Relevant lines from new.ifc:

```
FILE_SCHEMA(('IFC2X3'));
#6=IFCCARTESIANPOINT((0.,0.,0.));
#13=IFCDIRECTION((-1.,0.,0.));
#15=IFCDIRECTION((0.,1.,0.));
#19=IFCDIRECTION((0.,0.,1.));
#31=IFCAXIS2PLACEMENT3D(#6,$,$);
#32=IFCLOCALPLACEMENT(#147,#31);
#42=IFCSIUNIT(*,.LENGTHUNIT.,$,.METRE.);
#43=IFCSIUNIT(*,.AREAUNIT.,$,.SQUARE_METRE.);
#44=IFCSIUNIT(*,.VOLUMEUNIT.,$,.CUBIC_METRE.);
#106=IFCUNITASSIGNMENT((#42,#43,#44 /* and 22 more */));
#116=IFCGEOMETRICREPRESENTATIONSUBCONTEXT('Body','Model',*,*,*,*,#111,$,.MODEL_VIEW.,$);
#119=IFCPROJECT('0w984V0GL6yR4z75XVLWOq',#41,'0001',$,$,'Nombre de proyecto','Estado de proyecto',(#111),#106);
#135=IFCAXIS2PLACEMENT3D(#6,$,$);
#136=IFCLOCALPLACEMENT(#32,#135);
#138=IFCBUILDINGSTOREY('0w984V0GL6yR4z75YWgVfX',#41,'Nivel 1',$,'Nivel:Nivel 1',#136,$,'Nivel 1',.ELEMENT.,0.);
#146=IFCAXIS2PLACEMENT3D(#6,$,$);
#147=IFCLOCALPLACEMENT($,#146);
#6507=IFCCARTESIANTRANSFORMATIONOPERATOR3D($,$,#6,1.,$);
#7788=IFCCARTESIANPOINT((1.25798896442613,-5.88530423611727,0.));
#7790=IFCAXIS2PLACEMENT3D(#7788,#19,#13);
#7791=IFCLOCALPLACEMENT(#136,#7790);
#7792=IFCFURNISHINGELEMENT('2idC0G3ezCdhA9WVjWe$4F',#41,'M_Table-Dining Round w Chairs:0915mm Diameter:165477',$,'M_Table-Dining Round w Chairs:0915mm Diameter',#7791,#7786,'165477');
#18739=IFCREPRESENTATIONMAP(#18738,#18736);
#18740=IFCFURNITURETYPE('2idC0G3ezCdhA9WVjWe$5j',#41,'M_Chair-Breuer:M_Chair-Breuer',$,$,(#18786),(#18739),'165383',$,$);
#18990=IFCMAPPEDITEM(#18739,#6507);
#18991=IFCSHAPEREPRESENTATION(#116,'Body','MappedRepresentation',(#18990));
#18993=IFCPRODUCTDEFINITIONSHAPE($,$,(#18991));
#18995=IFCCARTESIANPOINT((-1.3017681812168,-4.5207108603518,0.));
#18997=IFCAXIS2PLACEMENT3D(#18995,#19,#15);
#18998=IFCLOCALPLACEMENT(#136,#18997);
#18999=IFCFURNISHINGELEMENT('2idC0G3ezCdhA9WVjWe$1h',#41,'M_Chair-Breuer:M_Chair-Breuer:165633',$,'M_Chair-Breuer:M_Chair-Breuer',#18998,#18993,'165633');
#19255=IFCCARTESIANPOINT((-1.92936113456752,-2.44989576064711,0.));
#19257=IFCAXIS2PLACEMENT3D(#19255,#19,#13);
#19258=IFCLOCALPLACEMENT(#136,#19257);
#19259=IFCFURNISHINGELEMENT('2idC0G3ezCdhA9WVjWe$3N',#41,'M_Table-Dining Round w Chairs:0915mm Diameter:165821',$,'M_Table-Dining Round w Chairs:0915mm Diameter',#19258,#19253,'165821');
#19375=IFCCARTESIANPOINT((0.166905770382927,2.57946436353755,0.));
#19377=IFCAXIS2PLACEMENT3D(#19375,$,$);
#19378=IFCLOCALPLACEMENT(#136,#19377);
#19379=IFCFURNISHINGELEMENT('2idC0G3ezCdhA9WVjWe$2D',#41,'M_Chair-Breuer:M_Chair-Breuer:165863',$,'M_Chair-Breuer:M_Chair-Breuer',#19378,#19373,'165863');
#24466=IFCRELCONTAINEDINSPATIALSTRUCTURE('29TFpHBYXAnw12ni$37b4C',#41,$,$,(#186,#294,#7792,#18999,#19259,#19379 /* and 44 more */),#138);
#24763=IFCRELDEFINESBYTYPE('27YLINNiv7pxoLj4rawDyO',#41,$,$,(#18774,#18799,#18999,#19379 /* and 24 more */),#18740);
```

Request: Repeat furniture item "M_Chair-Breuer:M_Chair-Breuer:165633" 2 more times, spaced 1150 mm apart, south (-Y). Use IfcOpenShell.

```python
import numpy as np
import ifcopenshell
import ifcopenshell.api.geometry
import ifcopenshell.api.root
import ifcopenshell.util.element
import ifcopenshell.util.placement

model = ifcopenshell.open("new.ifc")


def reuse_history(source, copy):
    """copy_class also copies each property set's owner history, people and application; keep the originals."""
    for rel in copy.IsDefinedBy:
        if rel.is_a("IfcRelDefinesByProperties") and (history := rel.RelatingPropertyDefinition.OwnerHistory):
            rel.RelatingPropertyDefinition.OwnerHistory = source.OwnerHistory
            ifcopenshell.util.element.remove_deep2(model, history)


source = model.by_guid("2idC0G3ezCdhA9WVjWe$1h")
base = ifcopenshell.util.placement.get_local_placement(source.ObjectPlacement)
step = np.array([0.0, -1.0, 0.0]) * 1.15

for i in range(1, 3):
    copy = ifcopenshell.api.root.copy_class(model, product=source)
    copy.Representation = ifcopenshell.util.element.copy_deep(
        model, source.Representation, exclude=["IfcGeometricRepresentationContext", "IfcRepresentationMap"]
    )
    copy.Name = "M_Chair-Breuer:M_Chair-Breuer"
    copy.Tag = None
    reuse_history(source, copy)
    matrix = base.copy()
    matrix[:3, 3] += i * step
    print("added at", matrix[:3, 3].round(3) + 0.0)
    ifcopenshell.api.geometry.edit_object_placement(model, product=copy, matrix=matrix, is_si=False)

model.write("new_updated.ifc")
```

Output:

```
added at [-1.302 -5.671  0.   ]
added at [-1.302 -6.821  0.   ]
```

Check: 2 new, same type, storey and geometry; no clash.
